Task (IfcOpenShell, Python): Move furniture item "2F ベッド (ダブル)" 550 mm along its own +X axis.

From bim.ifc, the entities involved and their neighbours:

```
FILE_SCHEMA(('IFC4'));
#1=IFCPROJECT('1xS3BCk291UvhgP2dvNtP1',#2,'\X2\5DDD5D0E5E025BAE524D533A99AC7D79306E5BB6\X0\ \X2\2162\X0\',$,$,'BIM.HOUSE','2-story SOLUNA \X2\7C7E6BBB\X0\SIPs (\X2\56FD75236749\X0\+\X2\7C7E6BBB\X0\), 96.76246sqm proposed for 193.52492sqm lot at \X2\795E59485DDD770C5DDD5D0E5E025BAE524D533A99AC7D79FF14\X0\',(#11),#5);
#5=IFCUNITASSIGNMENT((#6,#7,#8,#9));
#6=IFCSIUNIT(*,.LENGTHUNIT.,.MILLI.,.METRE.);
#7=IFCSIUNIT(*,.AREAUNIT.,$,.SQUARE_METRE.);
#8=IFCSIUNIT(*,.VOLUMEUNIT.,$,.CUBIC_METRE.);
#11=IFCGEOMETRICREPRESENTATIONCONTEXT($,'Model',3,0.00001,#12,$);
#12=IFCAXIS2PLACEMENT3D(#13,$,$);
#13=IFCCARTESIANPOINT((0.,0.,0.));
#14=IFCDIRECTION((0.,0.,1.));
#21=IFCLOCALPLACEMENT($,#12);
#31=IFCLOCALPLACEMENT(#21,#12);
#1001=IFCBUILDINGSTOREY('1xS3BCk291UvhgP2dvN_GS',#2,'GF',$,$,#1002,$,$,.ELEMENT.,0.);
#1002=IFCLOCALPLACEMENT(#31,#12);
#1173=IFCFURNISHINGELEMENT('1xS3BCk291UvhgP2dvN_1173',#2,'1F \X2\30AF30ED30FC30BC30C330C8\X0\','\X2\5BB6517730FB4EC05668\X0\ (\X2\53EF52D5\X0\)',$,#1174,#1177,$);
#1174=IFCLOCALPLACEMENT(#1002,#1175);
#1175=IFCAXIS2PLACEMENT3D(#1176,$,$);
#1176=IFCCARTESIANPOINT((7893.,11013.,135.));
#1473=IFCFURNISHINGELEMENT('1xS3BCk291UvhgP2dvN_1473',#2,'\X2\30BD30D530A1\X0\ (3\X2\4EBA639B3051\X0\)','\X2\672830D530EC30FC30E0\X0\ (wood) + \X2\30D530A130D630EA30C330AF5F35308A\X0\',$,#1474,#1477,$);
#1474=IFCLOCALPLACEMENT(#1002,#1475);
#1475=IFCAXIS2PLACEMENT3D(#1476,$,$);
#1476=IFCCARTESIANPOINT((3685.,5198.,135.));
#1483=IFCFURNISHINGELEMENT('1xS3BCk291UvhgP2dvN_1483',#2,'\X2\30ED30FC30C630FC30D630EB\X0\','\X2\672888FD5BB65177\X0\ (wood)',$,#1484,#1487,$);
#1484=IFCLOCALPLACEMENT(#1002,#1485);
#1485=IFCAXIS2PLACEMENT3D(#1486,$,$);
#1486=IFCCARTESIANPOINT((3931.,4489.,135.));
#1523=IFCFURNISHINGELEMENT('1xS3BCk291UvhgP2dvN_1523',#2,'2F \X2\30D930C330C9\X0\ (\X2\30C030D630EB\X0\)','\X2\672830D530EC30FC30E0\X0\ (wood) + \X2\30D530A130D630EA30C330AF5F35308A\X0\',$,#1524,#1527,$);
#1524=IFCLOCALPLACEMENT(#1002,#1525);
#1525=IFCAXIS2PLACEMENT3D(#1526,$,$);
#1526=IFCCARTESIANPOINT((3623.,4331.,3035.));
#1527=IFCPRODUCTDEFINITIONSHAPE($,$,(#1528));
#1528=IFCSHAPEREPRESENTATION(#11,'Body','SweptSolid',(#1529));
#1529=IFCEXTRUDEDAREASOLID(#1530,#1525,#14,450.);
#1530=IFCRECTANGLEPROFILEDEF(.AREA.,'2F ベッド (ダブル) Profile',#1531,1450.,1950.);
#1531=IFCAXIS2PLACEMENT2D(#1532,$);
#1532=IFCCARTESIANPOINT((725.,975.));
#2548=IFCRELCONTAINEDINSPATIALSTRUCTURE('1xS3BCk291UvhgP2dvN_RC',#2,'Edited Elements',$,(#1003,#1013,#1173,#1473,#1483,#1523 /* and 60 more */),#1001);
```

```python
import ifcopenshell
import ifcopenshell.api.geometry
import ifcopenshell.util.placement

model = ifcopenshell.open("bim.ifc")

item = model.by_guid("1xS3BCk291UvhgP2dvN_1523")
matrix = ifcopenshell.util.placement.get_local_placement(item.ObjectPlacement)
matrix[:3, 3] += matrix[:3, 0] * 550.0
ifcopenshell.api.geometry.edit_object_placement(model, product=item, matrix=matrix, is_si=False)

print(ifcopenshell.util.placement.get_local_placement(item.ObjectPlacement).round(3) + 0.0)

model.write("bim-out.ifc")
```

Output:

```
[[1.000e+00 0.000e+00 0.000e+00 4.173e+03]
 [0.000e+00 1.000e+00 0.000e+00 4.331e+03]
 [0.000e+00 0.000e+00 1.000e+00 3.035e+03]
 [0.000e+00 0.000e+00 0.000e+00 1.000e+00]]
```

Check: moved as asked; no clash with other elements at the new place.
